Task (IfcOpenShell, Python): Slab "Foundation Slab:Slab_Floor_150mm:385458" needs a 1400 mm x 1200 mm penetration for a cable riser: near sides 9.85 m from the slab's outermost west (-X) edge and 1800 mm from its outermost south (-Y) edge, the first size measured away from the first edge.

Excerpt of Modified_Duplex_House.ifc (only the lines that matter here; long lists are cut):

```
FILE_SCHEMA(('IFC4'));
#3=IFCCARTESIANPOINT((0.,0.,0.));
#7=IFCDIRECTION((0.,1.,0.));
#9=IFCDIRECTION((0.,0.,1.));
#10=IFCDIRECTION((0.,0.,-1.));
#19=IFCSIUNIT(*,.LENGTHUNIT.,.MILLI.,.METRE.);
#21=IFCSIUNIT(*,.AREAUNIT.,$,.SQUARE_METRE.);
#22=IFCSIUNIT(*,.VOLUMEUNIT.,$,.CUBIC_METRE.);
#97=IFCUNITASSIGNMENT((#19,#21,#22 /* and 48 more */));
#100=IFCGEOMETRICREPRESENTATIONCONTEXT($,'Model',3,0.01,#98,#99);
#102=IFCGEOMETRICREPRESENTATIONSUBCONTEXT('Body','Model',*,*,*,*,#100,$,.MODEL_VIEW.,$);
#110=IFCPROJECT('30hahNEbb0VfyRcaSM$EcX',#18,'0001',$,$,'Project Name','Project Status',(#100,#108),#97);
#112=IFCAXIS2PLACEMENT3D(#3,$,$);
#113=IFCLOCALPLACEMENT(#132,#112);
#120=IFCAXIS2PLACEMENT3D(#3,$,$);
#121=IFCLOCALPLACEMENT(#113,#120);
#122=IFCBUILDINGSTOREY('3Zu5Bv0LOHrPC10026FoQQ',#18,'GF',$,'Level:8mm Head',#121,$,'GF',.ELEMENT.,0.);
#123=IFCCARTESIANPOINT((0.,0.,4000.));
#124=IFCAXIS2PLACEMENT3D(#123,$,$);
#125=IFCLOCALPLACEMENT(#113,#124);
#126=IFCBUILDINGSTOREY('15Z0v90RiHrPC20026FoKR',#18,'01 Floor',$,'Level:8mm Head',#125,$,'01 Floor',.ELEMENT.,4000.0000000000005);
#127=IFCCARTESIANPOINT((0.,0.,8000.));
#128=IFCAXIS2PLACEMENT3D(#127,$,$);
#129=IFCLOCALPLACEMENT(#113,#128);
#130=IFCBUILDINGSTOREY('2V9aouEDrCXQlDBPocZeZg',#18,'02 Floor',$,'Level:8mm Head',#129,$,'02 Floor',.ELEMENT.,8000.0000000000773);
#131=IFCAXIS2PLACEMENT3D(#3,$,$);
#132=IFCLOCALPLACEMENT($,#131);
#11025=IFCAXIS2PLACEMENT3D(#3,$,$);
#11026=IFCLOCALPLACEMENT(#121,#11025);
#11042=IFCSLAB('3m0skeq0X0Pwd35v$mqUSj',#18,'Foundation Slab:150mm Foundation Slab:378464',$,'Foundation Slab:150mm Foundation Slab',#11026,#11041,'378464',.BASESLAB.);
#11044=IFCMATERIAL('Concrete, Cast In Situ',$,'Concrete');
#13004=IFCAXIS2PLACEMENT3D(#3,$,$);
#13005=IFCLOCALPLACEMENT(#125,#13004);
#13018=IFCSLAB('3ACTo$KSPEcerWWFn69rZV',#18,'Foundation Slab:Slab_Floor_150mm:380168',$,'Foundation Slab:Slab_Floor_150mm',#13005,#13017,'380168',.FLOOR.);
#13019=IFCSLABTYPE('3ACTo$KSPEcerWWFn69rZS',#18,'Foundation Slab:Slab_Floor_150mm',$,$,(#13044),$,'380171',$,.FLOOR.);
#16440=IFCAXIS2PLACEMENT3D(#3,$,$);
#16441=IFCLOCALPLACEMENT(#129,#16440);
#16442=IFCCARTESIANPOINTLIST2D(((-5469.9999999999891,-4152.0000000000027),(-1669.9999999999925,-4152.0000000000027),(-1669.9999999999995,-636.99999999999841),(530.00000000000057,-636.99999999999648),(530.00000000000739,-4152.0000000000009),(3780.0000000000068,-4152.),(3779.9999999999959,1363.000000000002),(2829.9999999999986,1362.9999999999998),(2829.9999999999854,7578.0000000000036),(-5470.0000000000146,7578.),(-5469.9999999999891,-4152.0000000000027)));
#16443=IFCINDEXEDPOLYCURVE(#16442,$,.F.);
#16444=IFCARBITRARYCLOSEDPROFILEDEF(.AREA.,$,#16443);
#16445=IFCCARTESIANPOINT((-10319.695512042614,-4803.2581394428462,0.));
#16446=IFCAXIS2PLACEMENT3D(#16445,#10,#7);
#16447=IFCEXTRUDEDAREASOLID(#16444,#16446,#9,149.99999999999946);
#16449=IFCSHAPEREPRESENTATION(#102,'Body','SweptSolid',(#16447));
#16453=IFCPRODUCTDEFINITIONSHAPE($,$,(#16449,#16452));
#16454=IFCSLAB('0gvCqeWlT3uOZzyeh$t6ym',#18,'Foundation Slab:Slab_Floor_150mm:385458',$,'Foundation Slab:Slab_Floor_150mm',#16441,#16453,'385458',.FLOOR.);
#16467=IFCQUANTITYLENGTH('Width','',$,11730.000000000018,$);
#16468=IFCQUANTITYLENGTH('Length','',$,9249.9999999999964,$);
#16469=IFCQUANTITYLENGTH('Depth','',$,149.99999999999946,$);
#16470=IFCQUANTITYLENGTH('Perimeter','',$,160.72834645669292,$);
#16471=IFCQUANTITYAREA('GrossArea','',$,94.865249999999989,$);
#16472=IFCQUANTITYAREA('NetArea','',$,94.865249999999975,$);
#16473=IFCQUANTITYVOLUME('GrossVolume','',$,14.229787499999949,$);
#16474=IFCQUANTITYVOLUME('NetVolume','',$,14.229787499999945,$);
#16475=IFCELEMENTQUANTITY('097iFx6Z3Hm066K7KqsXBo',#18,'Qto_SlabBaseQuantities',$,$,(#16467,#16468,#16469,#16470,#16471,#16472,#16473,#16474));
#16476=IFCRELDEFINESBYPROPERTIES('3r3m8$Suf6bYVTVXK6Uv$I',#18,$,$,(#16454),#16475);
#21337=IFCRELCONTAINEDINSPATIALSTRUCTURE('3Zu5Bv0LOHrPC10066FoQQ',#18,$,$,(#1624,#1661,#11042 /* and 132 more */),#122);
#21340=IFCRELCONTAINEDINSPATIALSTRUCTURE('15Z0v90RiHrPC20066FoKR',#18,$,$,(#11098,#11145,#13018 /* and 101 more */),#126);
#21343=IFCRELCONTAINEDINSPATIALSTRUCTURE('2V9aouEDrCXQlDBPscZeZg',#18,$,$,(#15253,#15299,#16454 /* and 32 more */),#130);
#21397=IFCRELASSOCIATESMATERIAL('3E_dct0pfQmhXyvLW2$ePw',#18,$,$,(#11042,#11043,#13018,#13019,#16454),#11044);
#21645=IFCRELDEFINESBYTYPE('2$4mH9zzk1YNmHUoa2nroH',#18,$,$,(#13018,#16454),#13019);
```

```python
import numpy as np
import ifcopenshell
import ifcopenshell.api.feature
import ifcopenshell.api.geometry
import ifcopenshell.api.pset
import ifcopenshell.api.root
import ifcopenshell.geom
import ifcopenshell.util.element
import ifcopenshell.util.placement
import ifcopenshell.util.representation
import ifcopenshell.util.shape
import ifcopenshell.util.unit

model = ifcopenshell.open("Modified_Duplex_House.ifc")
unit_scale = ifcopenshell.util.unit.calculate_unit_scale(model)
area_scale = ifcopenshell.util.unit.calculate_unit_scale(model, "AREAUNIT")
volume_scale = ifcopenshell.util.unit.calculate_unit_scale(model, "VOLUMEUNIT")
settings = ifcopenshell.geom.settings()


def volume(element):
    """Net volume in cubic metres, openings subtracted."""
    shape = ifcopenshell.geom.create_shape(settings, element)
    return ifcopenshell.util.shape.get_volume(shape.geometry)


slab = model.by_id(16454)
before = volume(slab)

# Extent in the slab's own axes, in metres. The edges named are its -X and -Y sides.
slab_shape = ifcopenshell.geom.create_shape(settings, slab)
vertices = ifcopenshell.util.shape.get_vertices(slab_shape.geometry)
x_min, y_min, bottom = vertices.min(axis=0)
top = vertices[:, 2].max()

opening = ifcopenshell.api.root.create_entity(model, ifc_class="IfcOpeningElement", name="Cable riser opening", predefined_type="OPENING")
context = ifcopenshell.util.representation.get_context(model, "Model", "Body", "MODEL_VIEW")
width, depth = 1.4, 1.2
outline = [(0.0, 0.0), (width, 0.0), (width, depth), (0.0, depth), (0.0, 0.0)]
# Overshoot both faces by 50 mm so the cut is clean.
shape = ifcopenshell.api.geometry.add_slab_representation(
    model, context=context, depth=top - bottom + 0.1, polyline=outline
)
ifcopenshell.api.geometry.assign_representation(model, product=opening, representation=shape)

matrix = ifcopenshell.util.placement.get_local_placement(slab.ObjectPlacement)
matrix[:, 3] = matrix @ np.append(np.array([x_min + 9.85, y_min + 1.8, bottom - 0.05]) / unit_scale, 1.0)
ifcopenshell.api.geometry.edit_object_placement(model, product=opening, matrix=matrix, is_si=False)
ifcopenshell.api.feature.add_feature(model, feature=opening, element=slab)

after = volume(slab)

# Update the slab's stored quantities.
qto = model.by_id(ifcopenshell.util.element.get_pset(slab, "Qto_SlabBaseQuantities", should_inherit=False)["id"])
ifcopenshell.api.pset.edit_qto(model, qto=qto, properties={
    "NetArea": after / (top - bottom) / area_scale,
    "NetVolume": after / volume_scale,
})

print(f"slab volume {before:.3f} -> {after:.3f} m3")

model.write("Modified_Duplex_House_v2.ifc")
```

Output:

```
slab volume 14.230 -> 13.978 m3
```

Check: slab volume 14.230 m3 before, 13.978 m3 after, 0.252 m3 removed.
